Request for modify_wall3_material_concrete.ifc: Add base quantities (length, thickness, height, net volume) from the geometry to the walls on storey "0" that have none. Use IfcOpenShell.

First a look at what the model holds.

```python
import ifcopenshell
import ifcopenshell.util.element
import ifcopenshell.util.unit

model = ifcopenshell.open("modify_wall3_material_concrete.ifc")
print(model.schema)
for unit_type in ("LENGTHUNIT", "AREAUNIT", "VOLUMEUNIT"):
    print(unit_type, ifcopenshell.util.unit.calculate_unit_scale(model, unit_type))
storey = next(s for s in model.by_type("IfcBuildingStorey") if s.Name == "0")
walls = [e for e in ifcopenshell.util.element.get_decomposition(storey) if e.is_a("IfcWall")]
for e in sorted(walls, key=lambda e: e.id()):
    print(e.id(), e.is_a(), e.Name, list(ifcopenshell.util.element.get_psets(e, qtos_only=True)), sep=" | ")
```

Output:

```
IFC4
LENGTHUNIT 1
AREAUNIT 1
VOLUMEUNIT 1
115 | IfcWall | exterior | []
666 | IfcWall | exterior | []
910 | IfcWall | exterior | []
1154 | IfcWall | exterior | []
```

```python
import ifcopenshell
import ifcopenshell.api.pset
import ifcopenshell.geom
import ifcopenshell.util.element
import ifcopenshell.util.shape
import ifcopenshell.util.unit

model = ifcopenshell.open("modify_wall3_material_concrete.ifc")
unit_scale = ifcopenshell.util.unit.calculate_unit_scale(model)
volume_scale = ifcopenshell.util.unit.calculate_unit_scale(model, "VOLUMEUNIT")
settings = ifcopenshell.geom.settings()

storey = next(s for s in model.by_type("IfcBuildingStorey") if s.Name == "0")
walls = [e for e in ifcopenshell.util.element.get_decomposition(storey) if e.is_a("IfcWall")]

for e in sorted(walls, key=lambda e: e.id()):
    if ifcopenshell.util.element.get_psets(e, qtos_only=True, should_inherit=False):
        continue
    # Geometry comes back in metres, in the element's own axes.
    shape = ifcopenshell.geom.create_shape(settings, e)
    values = {
        "Length": ifcopenshell.util.shape.get_x(shape.geometry) / unit_scale,
        "Width": ifcopenshell.util.shape.get_y(shape.geometry) / unit_scale,
        "Height": ifcopenshell.util.shape.get_z(shape.geometry) / unit_scale,
        "NetVolume": ifcopenshell.util.shape.get_volume(shape.geometry) / volume_scale,
    }
    qto = ifcopenshell.api.pset.add_qto(model, product=e, name="Qto_WallBaseQuantities")
    ifcopenshell.api.pset.edit_qto(model, qto=qto, properties=values)
    print(e.id(), {k: round(v, 3) for k, v in values.items()})

model.write("modify_wall3_material_concrete-out.ifc")
```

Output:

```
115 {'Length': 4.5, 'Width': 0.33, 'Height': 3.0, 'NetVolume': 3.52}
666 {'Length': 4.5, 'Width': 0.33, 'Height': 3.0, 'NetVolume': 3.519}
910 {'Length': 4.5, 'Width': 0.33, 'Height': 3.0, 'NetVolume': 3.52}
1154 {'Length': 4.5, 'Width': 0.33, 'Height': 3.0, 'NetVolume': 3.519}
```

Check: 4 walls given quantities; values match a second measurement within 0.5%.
